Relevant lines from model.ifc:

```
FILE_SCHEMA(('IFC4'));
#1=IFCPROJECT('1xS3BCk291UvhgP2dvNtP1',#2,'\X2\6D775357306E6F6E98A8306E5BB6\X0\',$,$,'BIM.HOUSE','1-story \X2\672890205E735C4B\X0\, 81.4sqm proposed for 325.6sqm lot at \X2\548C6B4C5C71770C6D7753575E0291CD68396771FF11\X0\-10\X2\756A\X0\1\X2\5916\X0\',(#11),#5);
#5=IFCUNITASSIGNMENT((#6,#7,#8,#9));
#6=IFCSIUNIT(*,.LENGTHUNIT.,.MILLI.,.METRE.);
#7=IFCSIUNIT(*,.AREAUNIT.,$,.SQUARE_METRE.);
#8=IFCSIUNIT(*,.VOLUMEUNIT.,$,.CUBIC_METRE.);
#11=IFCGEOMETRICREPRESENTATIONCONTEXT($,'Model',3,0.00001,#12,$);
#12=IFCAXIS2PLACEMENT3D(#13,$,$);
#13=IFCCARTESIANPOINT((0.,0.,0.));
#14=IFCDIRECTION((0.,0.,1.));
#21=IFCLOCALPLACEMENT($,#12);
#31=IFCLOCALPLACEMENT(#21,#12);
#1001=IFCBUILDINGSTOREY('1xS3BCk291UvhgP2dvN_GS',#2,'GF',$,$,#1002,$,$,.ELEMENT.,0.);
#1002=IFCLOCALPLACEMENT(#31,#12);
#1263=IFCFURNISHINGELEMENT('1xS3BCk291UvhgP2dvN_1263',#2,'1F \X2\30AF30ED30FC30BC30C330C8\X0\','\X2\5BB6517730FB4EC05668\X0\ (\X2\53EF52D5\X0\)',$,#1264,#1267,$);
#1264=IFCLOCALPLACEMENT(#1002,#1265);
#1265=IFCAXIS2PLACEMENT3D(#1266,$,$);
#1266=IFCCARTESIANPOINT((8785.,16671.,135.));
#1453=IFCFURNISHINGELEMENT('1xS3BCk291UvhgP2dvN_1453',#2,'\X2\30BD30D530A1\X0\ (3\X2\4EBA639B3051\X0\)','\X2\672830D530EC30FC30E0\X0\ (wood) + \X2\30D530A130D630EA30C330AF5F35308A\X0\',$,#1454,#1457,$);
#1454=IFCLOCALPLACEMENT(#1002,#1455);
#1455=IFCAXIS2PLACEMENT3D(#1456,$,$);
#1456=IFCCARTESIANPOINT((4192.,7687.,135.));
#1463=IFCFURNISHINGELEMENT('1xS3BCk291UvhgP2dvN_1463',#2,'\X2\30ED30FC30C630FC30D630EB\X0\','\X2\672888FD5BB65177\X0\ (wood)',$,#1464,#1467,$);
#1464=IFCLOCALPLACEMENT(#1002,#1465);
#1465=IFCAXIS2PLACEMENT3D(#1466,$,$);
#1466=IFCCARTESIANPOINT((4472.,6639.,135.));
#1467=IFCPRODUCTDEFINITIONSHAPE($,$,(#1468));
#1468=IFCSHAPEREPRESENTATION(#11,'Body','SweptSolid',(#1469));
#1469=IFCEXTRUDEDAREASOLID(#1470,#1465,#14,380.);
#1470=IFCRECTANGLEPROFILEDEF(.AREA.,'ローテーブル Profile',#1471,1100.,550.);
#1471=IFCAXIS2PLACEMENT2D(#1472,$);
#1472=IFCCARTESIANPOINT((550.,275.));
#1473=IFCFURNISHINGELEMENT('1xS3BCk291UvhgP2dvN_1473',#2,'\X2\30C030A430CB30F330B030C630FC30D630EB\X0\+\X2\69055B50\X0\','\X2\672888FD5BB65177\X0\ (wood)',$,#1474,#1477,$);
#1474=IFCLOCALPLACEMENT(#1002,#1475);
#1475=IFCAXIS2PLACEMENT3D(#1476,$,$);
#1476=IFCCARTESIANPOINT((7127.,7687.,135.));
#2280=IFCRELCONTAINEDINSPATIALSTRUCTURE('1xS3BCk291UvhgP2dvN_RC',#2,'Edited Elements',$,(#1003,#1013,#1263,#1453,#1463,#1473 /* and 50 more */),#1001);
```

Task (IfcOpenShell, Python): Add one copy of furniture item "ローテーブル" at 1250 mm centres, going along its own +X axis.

```python
import ifcopenshell
import ifcopenshell.api.geometry
import ifcopenshell.api.root
import ifcopenshell.util.element
import ifcopenshell.util.placement
import ifcopenshell.util.unit

model = ifcopenshell.open("model.ifc")
unit_scale = ifcopenshell.util.unit.calculate_unit_scale(model)


def reuse_history(source, copy):
    """copy_class also copies each property set's owner history, people and application; keep the originals."""
    for rel in copy.IsDefinedBy:
        if rel.is_a("IfcRelDefinesByProperties") and (history := rel.RelatingPropertyDefinition.OwnerHistory):
            rel.RelatingPropertyDefinition.OwnerHistory = source.OwnerHistory
            ifcopenshell.util.element.remove_deep2(model, history)


source = model.by_id(1463)
base = ifcopenshell.util.placement.get_local_placement(source.ObjectPlacement)
step = base[:3, 0] * 1.25 / unit_scale

for i in range(1, 2):
    copy = ifcopenshell.api.root.copy_class(model, product=source)
    copy.Representation = ifcopenshell.util.element.copy_deep(
        model, source.Representation, exclude=["IfcGeometricRepresentationContext", "IfcRepresentationMap"]
    )
    reuse_history(source, copy)
    matrix = base.copy()
    matrix[:3, 3] += i * step
    print("added at", matrix[:3, 3].round(3) + 0.0)
    ifcopenshell.api.geometry.edit_object_placement(model, product=copy, matrix=matrix, is_si=False)

model.write("model-out.ifc")
```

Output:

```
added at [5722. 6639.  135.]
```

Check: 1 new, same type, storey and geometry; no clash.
